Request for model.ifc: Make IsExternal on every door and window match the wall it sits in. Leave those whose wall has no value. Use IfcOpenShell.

First a look at what the model holds.

```python
import ifcopenshell
import ifcopenshell.util.element

model = ifcopenshell.open("model.ifc")
print(model.schema)
seen = {}
for e in model.by_type("IfcDoor") + model.by_type("IfcWindow"):
    if not e.FillsVoids:
        continue
    host = e.FillsVoids[0].RelatingOpeningElement.VoidsElements[0].RelatingBuildingElement
    own = ifcopenshell.util.element.get_pset(e, f"Pset_{e.is_a()[3:].removesuffix('StandardCase')}Common", "IsExternal")
    wall = ifcopenshell.util.element.get_pset(host, "Pset_WallCommon", "IsExternal")
    seen[e.is_a(), own, wall] = seen.get((e.is_a(), own, wall), 0) + 1
for (cls, own, wall), count in sorted(seen.items(), key=str):
    print(count, cls, "IsExternal:", own, "| host wall:", wall)
```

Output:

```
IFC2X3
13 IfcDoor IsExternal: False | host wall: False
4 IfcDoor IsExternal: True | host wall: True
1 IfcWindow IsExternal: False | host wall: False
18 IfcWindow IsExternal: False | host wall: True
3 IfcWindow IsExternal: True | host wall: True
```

```python
import ifcopenshell
import ifcopenshell.api.pset
import ifcopenshell.util.element

model = ifcopenshell.open("model.ifc")

count = 0
for ifc_class, pset_name in (("IfcDoor", "Pset_DoorCommon"), ("IfcWindow", "Pset_WindowCommon")):
    for e in model.by_type(ifc_class):
        if not e.FillsVoids:
            continue
        host = e.FillsVoids[0].RelatingOpeningElement.VoidsElements[0].RelatingBuildingElement
        external = ifcopenshell.util.element.get_pset(host, "Pset_WallCommon", "IsExternal")
        if external is None or ifcopenshell.util.element.get_pset(e, pset_name, "IsExternal") == external:
            continue
        pset = ifcopenshell.api.pset.add_pset(model, product=e, name=pset_name)
        ifcopenshell.api.pset.edit_pset(model, pset=pset, properties={"IsExternal": external})
        count += 1

print(count, "updated")

model.write("model_rev.ifc")
```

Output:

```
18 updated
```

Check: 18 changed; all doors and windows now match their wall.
